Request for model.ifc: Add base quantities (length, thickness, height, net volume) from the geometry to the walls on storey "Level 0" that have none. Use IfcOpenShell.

First a look at what the model holds.

```python
import ifcopenshell
import ifcopenshell.util.element
import ifcopenshell.util.unit

model = ifcopenshell.open("model.ifc")
print(model.schema)
for unit_type in ("LENGTHUNIT", "AREAUNIT", "VOLUMEUNIT"):
    print(unit_type, ifcopenshell.util.unit.calculate_unit_scale(model, unit_type))
storey = next(s for s in model.by_type("IfcBuildingStorey") if s.Name == "Level 0")
walls = [e for e in ifcopenshell.util.element.get_decomposition(storey) if e.is_a("IfcWall")]
for e in sorted(walls, key=lambda e: e.id()):
    print(e.id(), e.is_a(), e.Name, list(ifcopenshell.util.element.get_psets(e, qtos_only=True)), sep=" | ")
```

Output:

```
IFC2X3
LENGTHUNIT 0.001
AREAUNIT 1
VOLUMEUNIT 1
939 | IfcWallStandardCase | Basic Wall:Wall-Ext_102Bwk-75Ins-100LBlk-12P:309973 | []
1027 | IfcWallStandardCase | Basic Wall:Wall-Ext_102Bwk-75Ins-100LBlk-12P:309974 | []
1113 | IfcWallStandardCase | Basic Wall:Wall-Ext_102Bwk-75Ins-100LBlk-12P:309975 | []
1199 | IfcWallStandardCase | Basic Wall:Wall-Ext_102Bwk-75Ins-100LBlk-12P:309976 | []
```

```python
import ifcopenshell
import ifcopenshell.api.pset
import ifcopenshell.geom
import ifcopenshell.util.element
import ifcopenshell.util.shape
import ifcopenshell.util.unit

model = ifcopenshell.open("model.ifc")
unit_scale = ifcopenshell.util.unit.calculate_unit_scale(model)
volume_scale = ifcopenshell.util.unit.calculate_unit_scale(model, "VOLUMEUNIT")
settings = ifcopenshell.geom.settings()

storey = next(s for s in model.by_type("IfcBuildingStorey") if s.Name == "Level 0")
walls = [e for e in ifcopenshell.util.element.get_decomposition(storey) if e.is_a("IfcWall")]

for e in sorted(walls, key=lambda e: e.id()):
    if ifcopenshell.util.element.get_psets(e, qtos_only=True, should_inherit=False):
        continue
    # Geometry comes back in metres, in the element's own axes.
    shape = ifcopenshell.geom.create_shape(settings, e)
    values = {
        "Length": ifcopenshell.util.shape.get_x(shape.geometry) / unit_scale,
        "Width": ifcopenshell.util.shape.get_y(shape.geometry) / unit_scale,
        "Height": ifcopenshell.util.shape.get_z(shape.geometry) / unit_scale,
        "NetVolume": ifcopenshell.util.shape.get_volume(shape.geometry) / volume_scale,
    }
    qto = ifcopenshell.api.pset.add_qto(model, product=e, name="BaseQuantities")
    ifcopenshell.api.pset.edit_qto(model, qto=qto, properties=values)
    print(e.id(), {k: round(v, 3) for k, v in values.items()})

model.write("model-out.ifc")
```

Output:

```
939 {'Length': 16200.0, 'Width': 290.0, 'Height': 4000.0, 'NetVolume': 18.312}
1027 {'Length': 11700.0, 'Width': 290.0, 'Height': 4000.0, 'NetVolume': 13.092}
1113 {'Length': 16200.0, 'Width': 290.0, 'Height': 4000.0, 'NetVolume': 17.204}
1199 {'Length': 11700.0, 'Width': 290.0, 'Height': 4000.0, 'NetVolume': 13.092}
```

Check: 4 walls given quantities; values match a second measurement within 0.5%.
